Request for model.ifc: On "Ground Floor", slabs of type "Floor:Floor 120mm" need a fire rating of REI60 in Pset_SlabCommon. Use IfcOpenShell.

First a look at what the model holds.

```python
import ifcopenshell
import ifcopenshell.util.element

model = ifcopenshell.open("model.ifc")
print(model.schema)
storey = next(s for s in model.by_type("IfcBuildingStorey") if s.Name == "Ground Floor")
slabs = [e for e in ifcopenshell.util.element.get_decomposition(storey) if e.is_a("IfcSlab")]
seen = {}
for e in slabs:
    element_type = ifcopenshell.util.element.get_type(e)
    key = (element_type.Name if element_type != e and element_type else None, ifcopenshell.util.element.get_pset(e, "Pset_SlabCommon", "FireRating"))
    seen[key] = seen.get(key, 0) + 1
for (name, value), count in sorted(seen.items(), key=str):
    print(count, "x", name, "|", value)
```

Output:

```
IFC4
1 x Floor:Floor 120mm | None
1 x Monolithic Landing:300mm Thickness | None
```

```python
import ifcopenshell
import ifcopenshell.api.pset
import ifcopenshell.util.element

model = ifcopenshell.open("model.ifc")

storey = next(s for s in model.by_type("IfcBuildingStorey") if s.Name == "Ground Floor")
slabs = [e for e in ifcopenshell.util.element.get_decomposition(storey) if e.is_a("IfcSlab")]

count = 0
for e in slabs:
    element_type = ifcopenshell.util.element.get_type(e)
    if element_type in (None, e) or element_type.Name != "Floor:Floor 120mm":
        continue
    # add_pset returns the element's existing set when there is one.
    pset = ifcopenshell.api.pset.add_pset(model, product=e, name="Pset_SlabCommon")
    ifcopenshell.api.pset.edit_pset(model, pset=pset, properties={"FireRating": "REI60"})
    count += 1

print(count, "slabs updated")

model.write("model-out.ifc")
```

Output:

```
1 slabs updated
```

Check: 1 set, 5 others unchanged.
